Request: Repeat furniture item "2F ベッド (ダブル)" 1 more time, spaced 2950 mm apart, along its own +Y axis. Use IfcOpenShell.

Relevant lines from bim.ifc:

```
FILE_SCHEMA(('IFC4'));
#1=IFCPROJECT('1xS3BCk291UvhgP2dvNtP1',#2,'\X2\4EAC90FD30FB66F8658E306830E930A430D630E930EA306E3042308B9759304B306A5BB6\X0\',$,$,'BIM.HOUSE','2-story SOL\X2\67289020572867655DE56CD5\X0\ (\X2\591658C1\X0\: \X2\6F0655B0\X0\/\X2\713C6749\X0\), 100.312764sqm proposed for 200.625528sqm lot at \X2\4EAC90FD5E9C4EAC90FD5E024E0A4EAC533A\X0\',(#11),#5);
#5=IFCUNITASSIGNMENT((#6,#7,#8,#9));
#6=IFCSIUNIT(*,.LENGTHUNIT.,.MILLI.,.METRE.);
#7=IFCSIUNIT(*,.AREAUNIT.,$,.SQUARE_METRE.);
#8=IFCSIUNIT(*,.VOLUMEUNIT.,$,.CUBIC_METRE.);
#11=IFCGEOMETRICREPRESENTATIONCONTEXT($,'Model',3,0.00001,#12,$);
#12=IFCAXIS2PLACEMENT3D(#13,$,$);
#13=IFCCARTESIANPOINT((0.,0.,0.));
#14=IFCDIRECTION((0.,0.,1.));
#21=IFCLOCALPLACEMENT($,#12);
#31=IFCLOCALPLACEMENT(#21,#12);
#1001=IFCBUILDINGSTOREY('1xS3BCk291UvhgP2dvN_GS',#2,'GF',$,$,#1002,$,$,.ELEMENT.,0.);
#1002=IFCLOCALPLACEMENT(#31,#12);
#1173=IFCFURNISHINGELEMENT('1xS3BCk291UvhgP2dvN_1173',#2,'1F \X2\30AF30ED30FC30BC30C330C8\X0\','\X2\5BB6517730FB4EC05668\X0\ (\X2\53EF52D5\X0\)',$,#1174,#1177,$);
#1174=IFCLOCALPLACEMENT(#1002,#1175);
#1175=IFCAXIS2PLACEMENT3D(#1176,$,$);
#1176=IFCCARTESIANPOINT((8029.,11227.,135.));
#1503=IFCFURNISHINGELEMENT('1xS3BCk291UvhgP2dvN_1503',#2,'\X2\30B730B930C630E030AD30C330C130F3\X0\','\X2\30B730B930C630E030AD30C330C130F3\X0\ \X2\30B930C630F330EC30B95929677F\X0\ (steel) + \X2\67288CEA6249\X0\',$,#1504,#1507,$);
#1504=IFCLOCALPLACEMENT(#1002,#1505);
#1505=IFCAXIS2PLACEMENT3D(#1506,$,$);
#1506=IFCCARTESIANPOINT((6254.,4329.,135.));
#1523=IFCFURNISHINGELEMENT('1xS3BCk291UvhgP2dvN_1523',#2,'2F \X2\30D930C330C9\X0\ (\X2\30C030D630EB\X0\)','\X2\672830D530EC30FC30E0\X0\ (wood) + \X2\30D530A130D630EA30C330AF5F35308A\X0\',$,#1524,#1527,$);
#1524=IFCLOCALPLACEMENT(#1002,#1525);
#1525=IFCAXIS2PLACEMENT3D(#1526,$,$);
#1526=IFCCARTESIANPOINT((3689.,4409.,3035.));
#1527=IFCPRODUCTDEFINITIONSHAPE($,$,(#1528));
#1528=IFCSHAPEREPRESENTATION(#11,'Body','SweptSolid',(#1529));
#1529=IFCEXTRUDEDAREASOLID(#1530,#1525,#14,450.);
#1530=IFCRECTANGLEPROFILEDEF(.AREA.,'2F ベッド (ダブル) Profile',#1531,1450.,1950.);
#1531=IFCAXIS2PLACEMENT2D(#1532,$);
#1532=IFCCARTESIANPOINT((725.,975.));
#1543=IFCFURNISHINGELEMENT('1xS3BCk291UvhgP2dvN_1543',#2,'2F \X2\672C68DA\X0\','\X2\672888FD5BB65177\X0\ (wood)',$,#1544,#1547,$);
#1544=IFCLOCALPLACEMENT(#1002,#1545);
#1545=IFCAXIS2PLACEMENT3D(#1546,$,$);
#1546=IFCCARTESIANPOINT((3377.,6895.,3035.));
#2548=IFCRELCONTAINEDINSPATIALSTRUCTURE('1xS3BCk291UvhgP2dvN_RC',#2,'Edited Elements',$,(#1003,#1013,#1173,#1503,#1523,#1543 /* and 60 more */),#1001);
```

```python
import ifcopenshell
import ifcopenshell.api.geometry
import ifcopenshell.api.root
import ifcopenshell.util.element
import ifcopenshell.util.placement
import ifcopenshell.util.unit

model = ifcopenshell.open("bim.ifc")
unit_scale = ifcopenshell.util.unit.calculate_unit_scale(model)


def reuse_history(source, copy):
    """copy_class also copies each property set's owner history, people and application; keep the originals."""
    for rel in copy.IsDefinedBy:
        if rel.is_a("IfcRelDefinesByProperties") and (history := rel.RelatingPropertyDefinition.OwnerHistory):
            rel.RelatingPropertyDefinition.OwnerHistory = source.OwnerHistory
            ifcopenshell.util.element.remove_deep2(model, history)


source = model.by_guid("1xS3BCk291UvhgP2dvN_1523")
base = ifcopenshell.util.placement.get_local_placement(source.ObjectPlacement)
step = base[:3, 1] * 2.95 / unit_scale

for i in range(1, 2):
    copy = ifcopenshell.api.root.copy_class(model, product=source)
    copy.Representation = ifcopenshell.util.element.copy_deep(
        model, source.Representation, exclude=["IfcGeometricRepresentationContext", "IfcRepresentationMap"]
    )
    reuse_history(source, copy)
    matrix = base.copy()
    matrix[:3, 3] += i * step
    print("added at", matrix[:3, 3].round(3) + 0.0)
    ifcopenshell.api.geometry.edit_object_placement(model, product=copy, matrix=matrix, is_si=False)

model.write("bim_edited.ifc")
```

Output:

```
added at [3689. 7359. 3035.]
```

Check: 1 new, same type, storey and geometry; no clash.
